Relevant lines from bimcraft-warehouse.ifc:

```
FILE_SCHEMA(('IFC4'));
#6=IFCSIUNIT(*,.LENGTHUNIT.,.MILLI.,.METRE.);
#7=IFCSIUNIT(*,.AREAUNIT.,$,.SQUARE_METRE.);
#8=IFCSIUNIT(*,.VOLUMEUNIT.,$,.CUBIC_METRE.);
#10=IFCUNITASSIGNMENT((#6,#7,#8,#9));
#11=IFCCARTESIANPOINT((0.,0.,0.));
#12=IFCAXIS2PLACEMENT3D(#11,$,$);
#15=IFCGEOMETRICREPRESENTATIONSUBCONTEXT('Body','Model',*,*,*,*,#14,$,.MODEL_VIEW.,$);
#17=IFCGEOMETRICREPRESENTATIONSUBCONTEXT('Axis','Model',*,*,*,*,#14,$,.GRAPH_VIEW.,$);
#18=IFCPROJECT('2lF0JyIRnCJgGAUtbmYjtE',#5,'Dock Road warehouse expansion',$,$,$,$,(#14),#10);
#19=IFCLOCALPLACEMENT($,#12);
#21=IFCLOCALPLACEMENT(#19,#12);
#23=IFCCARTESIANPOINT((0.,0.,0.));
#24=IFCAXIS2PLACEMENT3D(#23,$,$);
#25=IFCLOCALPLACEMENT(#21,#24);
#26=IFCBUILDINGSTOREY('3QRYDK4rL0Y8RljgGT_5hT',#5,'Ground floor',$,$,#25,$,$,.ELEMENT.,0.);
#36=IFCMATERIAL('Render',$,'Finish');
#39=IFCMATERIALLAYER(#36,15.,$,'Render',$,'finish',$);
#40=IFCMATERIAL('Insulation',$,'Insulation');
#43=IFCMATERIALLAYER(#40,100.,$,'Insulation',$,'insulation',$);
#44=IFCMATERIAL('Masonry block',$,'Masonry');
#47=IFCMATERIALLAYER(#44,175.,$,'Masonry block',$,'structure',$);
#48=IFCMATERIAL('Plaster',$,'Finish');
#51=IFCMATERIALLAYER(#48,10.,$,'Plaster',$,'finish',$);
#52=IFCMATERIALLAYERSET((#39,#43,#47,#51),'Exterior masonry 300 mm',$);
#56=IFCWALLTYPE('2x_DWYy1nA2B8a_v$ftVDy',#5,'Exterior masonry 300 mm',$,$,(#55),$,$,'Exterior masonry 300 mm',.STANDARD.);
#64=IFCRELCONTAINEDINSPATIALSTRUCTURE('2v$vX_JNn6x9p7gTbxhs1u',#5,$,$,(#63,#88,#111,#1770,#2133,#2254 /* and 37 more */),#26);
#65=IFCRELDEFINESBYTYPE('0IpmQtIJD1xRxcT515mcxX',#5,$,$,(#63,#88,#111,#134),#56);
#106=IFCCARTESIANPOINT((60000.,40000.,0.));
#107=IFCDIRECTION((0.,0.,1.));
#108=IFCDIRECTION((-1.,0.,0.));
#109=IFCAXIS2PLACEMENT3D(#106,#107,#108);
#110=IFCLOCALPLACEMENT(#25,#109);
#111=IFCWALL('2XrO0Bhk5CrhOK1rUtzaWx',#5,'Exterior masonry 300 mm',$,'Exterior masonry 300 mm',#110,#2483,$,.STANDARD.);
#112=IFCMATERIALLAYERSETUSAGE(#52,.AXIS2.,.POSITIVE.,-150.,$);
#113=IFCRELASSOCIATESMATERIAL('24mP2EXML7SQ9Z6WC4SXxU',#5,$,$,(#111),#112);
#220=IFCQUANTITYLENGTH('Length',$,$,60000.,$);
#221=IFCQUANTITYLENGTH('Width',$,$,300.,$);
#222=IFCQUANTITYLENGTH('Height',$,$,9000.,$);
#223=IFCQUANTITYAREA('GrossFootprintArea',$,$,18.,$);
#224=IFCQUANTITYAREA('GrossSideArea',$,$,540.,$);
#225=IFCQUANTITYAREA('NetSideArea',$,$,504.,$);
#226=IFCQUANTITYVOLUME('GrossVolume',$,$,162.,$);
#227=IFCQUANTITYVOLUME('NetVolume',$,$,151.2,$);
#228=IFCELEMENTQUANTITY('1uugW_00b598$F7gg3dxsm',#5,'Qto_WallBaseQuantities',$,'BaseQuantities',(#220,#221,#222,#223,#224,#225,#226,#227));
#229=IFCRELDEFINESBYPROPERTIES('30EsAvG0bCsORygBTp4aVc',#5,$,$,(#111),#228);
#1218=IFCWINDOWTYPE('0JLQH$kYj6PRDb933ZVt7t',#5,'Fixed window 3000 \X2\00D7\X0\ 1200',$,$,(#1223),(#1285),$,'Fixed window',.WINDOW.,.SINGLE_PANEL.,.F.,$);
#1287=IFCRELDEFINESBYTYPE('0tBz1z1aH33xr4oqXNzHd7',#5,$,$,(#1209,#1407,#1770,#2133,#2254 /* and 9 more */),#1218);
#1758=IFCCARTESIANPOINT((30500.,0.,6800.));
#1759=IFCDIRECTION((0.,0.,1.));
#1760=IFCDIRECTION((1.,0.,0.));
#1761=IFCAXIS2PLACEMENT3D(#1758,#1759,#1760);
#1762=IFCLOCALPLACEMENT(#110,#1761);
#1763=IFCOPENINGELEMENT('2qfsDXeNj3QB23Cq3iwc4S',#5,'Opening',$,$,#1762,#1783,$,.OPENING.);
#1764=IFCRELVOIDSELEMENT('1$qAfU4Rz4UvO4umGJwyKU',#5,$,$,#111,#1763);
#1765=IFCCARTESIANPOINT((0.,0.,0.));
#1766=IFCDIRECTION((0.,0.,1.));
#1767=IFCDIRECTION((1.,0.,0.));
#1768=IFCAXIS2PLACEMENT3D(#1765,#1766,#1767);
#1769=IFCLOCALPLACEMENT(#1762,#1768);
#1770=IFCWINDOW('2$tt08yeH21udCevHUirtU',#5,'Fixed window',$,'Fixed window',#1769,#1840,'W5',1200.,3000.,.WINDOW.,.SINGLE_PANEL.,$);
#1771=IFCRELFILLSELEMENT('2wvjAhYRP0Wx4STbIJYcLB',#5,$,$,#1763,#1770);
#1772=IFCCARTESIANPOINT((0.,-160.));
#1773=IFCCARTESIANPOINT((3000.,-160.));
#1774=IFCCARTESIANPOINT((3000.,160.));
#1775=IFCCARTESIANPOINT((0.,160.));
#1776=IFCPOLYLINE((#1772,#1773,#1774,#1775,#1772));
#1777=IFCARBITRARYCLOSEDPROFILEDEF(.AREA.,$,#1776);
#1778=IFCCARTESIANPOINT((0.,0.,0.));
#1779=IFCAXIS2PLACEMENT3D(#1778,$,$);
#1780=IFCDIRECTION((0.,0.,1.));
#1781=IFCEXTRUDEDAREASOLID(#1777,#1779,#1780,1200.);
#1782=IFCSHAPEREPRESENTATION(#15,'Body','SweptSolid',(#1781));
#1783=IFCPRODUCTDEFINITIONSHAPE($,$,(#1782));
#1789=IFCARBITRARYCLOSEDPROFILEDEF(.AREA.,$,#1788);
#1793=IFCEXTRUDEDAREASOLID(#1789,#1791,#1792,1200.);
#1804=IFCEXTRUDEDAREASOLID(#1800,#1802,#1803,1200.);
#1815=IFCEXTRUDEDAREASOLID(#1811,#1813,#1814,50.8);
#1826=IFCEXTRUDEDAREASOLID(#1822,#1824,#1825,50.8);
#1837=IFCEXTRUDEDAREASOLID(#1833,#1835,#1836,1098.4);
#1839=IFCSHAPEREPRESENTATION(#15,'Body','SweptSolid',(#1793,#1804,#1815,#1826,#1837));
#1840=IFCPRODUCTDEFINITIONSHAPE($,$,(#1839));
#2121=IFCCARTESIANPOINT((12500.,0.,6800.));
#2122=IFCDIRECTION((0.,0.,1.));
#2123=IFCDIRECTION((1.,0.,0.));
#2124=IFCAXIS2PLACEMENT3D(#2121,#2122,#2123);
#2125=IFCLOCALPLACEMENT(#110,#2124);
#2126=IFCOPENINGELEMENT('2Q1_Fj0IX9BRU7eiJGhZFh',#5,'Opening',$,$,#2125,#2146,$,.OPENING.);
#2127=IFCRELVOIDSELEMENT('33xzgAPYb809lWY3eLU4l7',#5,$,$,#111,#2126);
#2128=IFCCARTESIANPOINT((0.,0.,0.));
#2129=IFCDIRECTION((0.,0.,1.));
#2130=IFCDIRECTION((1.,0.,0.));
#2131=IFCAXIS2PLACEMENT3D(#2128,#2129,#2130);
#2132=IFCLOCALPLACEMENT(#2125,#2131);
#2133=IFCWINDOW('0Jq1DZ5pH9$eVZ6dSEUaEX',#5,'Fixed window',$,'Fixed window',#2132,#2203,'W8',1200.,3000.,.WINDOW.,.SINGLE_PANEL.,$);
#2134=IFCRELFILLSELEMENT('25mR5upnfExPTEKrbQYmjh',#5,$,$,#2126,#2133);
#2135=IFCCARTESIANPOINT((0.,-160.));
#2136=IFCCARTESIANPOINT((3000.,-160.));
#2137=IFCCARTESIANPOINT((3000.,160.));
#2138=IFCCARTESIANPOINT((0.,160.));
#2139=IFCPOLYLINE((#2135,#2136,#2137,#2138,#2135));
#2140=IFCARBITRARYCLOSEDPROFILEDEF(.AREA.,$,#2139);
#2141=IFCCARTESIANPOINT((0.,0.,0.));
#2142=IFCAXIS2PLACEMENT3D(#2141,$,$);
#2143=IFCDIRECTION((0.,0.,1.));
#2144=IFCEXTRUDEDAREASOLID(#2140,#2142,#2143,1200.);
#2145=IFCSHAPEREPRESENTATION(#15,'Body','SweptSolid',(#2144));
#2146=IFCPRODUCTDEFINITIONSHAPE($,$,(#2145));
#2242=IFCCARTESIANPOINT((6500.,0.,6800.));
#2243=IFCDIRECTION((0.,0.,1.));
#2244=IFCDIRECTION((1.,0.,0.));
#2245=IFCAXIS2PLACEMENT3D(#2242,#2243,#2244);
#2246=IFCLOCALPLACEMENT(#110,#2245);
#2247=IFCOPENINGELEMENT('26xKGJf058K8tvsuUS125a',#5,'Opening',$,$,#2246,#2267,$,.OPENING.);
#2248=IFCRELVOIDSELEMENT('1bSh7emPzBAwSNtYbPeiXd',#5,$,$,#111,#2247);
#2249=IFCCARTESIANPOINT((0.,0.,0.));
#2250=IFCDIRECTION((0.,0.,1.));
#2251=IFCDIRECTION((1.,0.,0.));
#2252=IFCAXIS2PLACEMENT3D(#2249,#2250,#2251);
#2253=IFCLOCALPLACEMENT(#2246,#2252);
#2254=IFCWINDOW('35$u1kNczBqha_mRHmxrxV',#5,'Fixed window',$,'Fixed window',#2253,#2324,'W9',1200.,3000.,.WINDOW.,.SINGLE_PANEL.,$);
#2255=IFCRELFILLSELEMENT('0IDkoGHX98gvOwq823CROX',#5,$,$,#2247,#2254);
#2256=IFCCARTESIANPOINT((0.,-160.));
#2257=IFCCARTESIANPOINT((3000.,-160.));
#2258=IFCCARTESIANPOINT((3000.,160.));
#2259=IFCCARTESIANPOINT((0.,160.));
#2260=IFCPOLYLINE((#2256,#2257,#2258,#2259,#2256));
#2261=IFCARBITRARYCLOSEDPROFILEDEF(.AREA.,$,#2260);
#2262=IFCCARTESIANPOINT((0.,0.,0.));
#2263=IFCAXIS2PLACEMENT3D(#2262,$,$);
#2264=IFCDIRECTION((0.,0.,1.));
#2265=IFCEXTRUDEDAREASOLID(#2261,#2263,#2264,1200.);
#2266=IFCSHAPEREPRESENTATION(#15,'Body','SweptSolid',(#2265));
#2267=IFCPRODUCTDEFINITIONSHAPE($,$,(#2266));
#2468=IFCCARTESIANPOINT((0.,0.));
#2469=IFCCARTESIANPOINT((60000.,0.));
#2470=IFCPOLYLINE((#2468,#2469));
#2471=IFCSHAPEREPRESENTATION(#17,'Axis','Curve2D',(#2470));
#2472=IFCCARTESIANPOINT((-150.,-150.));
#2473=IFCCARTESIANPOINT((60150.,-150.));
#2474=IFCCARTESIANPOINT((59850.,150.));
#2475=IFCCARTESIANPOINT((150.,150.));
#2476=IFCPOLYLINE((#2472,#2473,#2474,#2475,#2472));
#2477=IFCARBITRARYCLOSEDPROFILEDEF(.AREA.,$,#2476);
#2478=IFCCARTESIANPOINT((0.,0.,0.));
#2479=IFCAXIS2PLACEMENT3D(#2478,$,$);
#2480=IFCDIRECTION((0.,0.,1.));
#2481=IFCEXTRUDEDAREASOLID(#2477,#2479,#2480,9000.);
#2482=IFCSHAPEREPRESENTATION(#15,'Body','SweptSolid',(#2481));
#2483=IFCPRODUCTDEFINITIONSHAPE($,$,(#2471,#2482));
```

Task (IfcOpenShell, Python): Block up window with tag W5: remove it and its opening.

```python
import ifcopenshell
import ifcopenshell.api.feature
import ifcopenshell.api.pset
import ifcopenshell.api.root
import ifcopenshell.geom
import ifcopenshell.util.element
import ifcopenshell.util.shape
import ifcopenshell.util.unit

model = ifcopenshell.open("bimcraft-warehouse.ifc")
area_scale = ifcopenshell.util.unit.calculate_unit_scale(model, "AREAUNIT")
volume_scale = ifcopenshell.util.unit.calculate_unit_scale(model, "VOLUMEUNIT")
settings = ifcopenshell.geom.settings()


def volume(element):
    """Net volume in cubic metres, openings subtracted."""
    shape = ifcopenshell.geom.create_shape(settings, element)
    return ifcopenshell.util.shape.get_volume(shape.geometry)


window = model.by_guid("2$tt08yeH21udCevHUirtU")
opening = window.FillsVoids[0].RelatingOpeningElement
wall = opening.VoidsElements[0].RelatingBuildingElement
before = volume(wall)

ifcopenshell.api.root.remove_product(model, product=window)
ifcopenshell.api.feature.remove_feature(model, feature=opening)

after = volume(wall)
thickness = 0.3  # wall thickness in metres

# Update the wall's stored quantities.
qto = model.by_id(ifcopenshell.util.element.get_pset(wall, "Qto_WallBaseQuantities", should_inherit=False)["id"])
ifcopenshell.api.pset.edit_qto(model, qto=qto, properties={
    "NetSideArea": after / thickness / area_scale,
    "NetVolume": after / volume_scale,
})

print(f"wall volume {before:.3f} -> {after:.3f} m3")

model.write("bimcraft-warehouse_updated.ifc")
```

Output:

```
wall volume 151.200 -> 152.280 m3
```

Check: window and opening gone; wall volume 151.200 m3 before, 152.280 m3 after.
